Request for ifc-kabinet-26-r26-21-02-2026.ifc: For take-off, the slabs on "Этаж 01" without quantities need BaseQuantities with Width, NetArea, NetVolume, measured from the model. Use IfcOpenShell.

First a look at what the model holds.

```python
import ifcopenshell
import ifcopenshell.util.element
import ifcopenshell.util.unit

model = ifcopenshell.open("ifc-kabinet-26-r26-21-02-2026.ifc")
print(model.schema)
for unit_type in ("LENGTHUNIT", "AREAUNIT", "VOLUMEUNIT"):
    print(unit_type, ifcopenshell.util.unit.calculate_unit_scale(model, unit_type))
storey = next(s for s in model.by_type("IfcBuildingStorey") if s.Name == "Этаж 01")
slabs = [e for e in ifcopenshell.util.element.get_decomposition(storey) if e.is_a("IfcSlab")]
for e in sorted(slabs, key=lambda e: e.id()):
    print(e.id(), e.is_a(), e.Name, list(ifcopenshell.util.element.get_psets(e, qtos_only=True)), sep=" | ")
```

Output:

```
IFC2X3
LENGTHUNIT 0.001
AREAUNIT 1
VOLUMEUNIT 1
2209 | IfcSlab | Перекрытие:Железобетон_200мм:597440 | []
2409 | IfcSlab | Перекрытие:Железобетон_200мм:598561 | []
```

```python
import ifcopenshell
import ifcopenshell.api.pset
import ifcopenshell.geom
import ifcopenshell.util.element
import ifcopenshell.util.shape
import ifcopenshell.util.unit

model = ifcopenshell.open("ifc-kabinet-26-r26-21-02-2026.ifc")
unit_scale = ifcopenshell.util.unit.calculate_unit_scale(model)
area_scale = ifcopenshell.util.unit.calculate_unit_scale(model, "AREAUNIT")
volume_scale = ifcopenshell.util.unit.calculate_unit_scale(model, "VOLUMEUNIT")
settings = ifcopenshell.geom.settings()

storey = next(s for s in model.by_type("IfcBuildingStorey") if s.Name == "Этаж 01")
slabs = [e for e in ifcopenshell.util.element.get_decomposition(storey) if e.is_a("IfcSlab")]

for e in sorted(slabs, key=lambda e: e.id()):
    if ifcopenshell.util.element.get_psets(e, qtos_only=True, should_inherit=False):
        continue
    # Geometry comes back in metres, in the element's own axes.
    shape = ifcopenshell.geom.create_shape(settings, e)
    values = {
        "Width": ifcopenshell.util.shape.get_z(shape.geometry) / unit_scale,
        "NetArea": ifcopenshell.util.shape.get_footprint_area(shape.geometry) / area_scale,
        "NetVolume": ifcopenshell.util.shape.get_volume(shape.geometry) / volume_scale,
    }
    qto = ifcopenshell.api.pset.add_qto(model, product=e, name="BaseQuantities")
    ifcopenshell.api.pset.edit_qto(model, qto=qto, properties=values)
    print(e.id(), {k: round(v, 3) for k, v in values.items()})

model.write("ifc-kabinet-26-r26-21-02-2026_edited.ifc")
```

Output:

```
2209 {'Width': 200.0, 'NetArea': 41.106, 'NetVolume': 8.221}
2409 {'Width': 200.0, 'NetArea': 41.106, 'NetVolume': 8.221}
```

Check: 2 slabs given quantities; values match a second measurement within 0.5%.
